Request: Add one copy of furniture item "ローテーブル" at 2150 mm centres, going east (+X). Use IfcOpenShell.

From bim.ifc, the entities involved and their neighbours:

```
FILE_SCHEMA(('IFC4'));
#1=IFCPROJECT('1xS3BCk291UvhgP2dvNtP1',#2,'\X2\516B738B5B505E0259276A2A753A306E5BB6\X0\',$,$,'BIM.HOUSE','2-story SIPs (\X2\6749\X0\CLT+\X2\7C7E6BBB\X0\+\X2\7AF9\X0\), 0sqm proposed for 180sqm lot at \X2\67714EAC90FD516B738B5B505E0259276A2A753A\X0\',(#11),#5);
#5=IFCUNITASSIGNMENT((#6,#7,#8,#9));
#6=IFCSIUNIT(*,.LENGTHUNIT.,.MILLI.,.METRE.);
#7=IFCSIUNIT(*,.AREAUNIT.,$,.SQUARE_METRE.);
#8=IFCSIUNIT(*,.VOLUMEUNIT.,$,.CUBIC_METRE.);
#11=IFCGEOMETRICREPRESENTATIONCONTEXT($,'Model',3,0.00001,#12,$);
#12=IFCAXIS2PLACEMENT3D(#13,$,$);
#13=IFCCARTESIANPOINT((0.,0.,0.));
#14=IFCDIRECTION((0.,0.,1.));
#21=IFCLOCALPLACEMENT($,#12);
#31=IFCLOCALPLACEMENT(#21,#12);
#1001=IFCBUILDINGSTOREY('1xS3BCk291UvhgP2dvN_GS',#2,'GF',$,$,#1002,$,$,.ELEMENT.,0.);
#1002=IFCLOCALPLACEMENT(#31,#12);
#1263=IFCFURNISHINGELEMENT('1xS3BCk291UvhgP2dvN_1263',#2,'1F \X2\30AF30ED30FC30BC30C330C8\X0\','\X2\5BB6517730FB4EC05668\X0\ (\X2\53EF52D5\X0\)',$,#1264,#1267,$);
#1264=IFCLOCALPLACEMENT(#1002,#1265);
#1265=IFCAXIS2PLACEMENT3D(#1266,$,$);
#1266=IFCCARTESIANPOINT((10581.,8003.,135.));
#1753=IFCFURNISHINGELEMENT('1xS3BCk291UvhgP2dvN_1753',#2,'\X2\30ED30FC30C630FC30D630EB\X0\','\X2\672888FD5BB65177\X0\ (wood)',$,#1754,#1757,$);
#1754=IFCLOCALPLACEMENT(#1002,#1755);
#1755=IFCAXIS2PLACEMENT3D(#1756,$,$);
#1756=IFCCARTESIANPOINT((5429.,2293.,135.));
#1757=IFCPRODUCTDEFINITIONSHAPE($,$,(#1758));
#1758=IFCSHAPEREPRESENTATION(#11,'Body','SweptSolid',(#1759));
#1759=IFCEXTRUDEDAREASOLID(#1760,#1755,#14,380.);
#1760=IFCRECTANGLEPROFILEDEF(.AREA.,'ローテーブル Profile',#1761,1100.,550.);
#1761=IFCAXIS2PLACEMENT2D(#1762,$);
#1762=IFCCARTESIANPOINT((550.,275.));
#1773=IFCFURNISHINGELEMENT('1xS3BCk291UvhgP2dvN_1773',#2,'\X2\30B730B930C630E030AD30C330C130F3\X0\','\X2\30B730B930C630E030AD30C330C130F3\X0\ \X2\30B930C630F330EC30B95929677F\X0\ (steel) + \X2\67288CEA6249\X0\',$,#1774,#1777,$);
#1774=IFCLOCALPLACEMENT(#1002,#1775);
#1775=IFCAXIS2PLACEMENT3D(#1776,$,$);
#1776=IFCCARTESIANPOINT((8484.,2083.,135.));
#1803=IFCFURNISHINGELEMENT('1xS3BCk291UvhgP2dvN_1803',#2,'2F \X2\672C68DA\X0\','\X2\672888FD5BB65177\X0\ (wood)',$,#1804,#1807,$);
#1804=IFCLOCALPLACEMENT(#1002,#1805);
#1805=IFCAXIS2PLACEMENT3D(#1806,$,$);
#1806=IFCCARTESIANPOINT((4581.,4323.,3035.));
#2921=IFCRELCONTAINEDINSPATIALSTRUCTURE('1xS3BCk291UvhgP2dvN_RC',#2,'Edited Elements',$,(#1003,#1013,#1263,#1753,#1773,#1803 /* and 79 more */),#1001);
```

```python
import numpy as np
import ifcopenshell
import ifcopenshell.api.geometry
import ifcopenshell.api.root
import ifcopenshell.util.element
import ifcopenshell.util.placement

model = ifcopenshell.open("bim.ifc")


def reuse_history(source, copy):
    """copy_class also copies each property set's owner history, people and application; keep the originals."""
    for rel in copy.IsDefinedBy:
        if rel.is_a("IfcRelDefinesByProperties") and (history := rel.RelatingPropertyDefinition.OwnerHistory):
            rel.RelatingPropertyDefinition.OwnerHistory = source.OwnerHistory
            ifcopenshell.util.element.remove_deep2(model, history)


source = model.by_guid("1xS3BCk291UvhgP2dvN_1753")
base = ifcopenshell.util.placement.get_local_placement(source.ObjectPlacement)
step = np.array([1.0, 0.0, 0.0]) * 2150.0

for i in range(1, 2):
    copy = ifcopenshell.api.root.copy_class(model, product=source)
    copy.Representation = ifcopenshell.util.element.copy_deep(
        model, source.Representation, exclude=["IfcGeometricRepresentationContext", "IfcRepresentationMap"]
    )
    reuse_history(source, copy)
    matrix = base.copy()
    matrix[:3, 3] += i * step
    print("added at", matrix[:3, 3].round(3) + 0.0)
    ifcopenshell.api.geometry.edit_object_placement(model, product=copy, matrix=matrix, is_si=False)

model.write("bim_rev.ifc")
```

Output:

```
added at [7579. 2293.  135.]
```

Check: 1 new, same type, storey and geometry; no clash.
